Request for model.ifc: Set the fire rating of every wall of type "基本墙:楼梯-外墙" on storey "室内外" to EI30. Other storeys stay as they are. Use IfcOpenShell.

First a look at what the model holds.

```python
import ifcopenshell
import ifcopenshell.util.element

model = ifcopenshell.open("model.ifc")
print(model.schema)
storey = next(s for s in model.by_type("IfcBuildingStorey") if s.Name == "室内外")
walls = [e for e in ifcopenshell.util.element.get_decomposition(storey) if e.is_a("IfcWall")]
seen = {}
for e in walls:
    element_type = ifcopenshell.util.element.get_type(e)
    key = (element_type.Name if element_type != e and element_type else None, ifcopenshell.util.element.get_pset(e, "Pset_WallCommon", "FireRating"))
    seen[key] = seen.get(key, 0) + 1
for (name, value), count in sorted(seen.items(), key=str):
    print(count, "x", name, "|", value)
```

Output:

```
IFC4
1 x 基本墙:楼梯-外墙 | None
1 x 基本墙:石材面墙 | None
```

```python
import ifcopenshell
import ifcopenshell.api.pset
import ifcopenshell.util.element

model = ifcopenshell.open("model.ifc")

storey = next(s for s in model.by_type("IfcBuildingStorey") if s.Name == "室内外")
walls = [e for e in ifcopenshell.util.element.get_decomposition(storey) if e.is_a("IfcWall")]

count = 0
for e in walls:
    element_type = ifcopenshell.util.element.get_type(e)
    if element_type in (None, e) or element_type.Name != "基本墙:楼梯-外墙":
        continue
    # add_pset returns the element's existing set when there is one.
    pset = ifcopenshell.api.pset.add_pset(model, product=e, name="Pset_WallCommon")
    ifcopenshell.api.pset.edit_pset(model, pset=pset, properties={"FireRating": "EI30"})
    count += 1

print(count, "walls updated")

model.write("model-out.ifc")
```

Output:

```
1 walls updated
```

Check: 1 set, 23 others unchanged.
